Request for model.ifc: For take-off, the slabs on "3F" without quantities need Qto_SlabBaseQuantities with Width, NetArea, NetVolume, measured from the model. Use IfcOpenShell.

First a look at what the model holds.

```python
import ifcopenshell
import ifcopenshell.util.element
import ifcopenshell.util.unit

model = ifcopenshell.open("model.ifc")
print(model.schema)
for unit_type in ("LENGTHUNIT", "AREAUNIT", "VOLUMEUNIT"):
    print(unit_type, ifcopenshell.util.unit.calculate_unit_scale(model, unit_type))
storey = next(s for s in model.by_type("IfcBuildingStorey") if s.Name == "3F")
slabs = [e for e in ifcopenshell.util.element.get_decomposition(storey) if e.is_a("IfcSlab")]
for e in sorted(slabs, key=lambda e: e.id()):
    print(e.id(), e.is_a(), e.Name, list(ifcopenshell.util.element.get_psets(e, qtos_only=True)), sep=" | ")
```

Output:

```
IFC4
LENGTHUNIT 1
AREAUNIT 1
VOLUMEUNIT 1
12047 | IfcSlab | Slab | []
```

```python
import ifcopenshell
import ifcopenshell.api.pset
import ifcopenshell.geom
import ifcopenshell.util.element
import ifcopenshell.util.shape
import ifcopenshell.util.unit

model = ifcopenshell.open("model.ifc")
unit_scale = ifcopenshell.util.unit.calculate_unit_scale(model)
area_scale = ifcopenshell.util.unit.calculate_unit_scale(model, "AREAUNIT")
volume_scale = ifcopenshell.util.unit.calculate_unit_scale(model, "VOLUMEUNIT")
settings = ifcopenshell.geom.settings()

storey = next(s for s in model.by_type("IfcBuildingStorey") if s.Name == "3F")
slabs = [e for e in ifcopenshell.util.element.get_decomposition(storey) if e.is_a("IfcSlab")]

for e in sorted(slabs, key=lambda e: e.id()):
    if ifcopenshell.util.element.get_psets(e, qtos_only=True, should_inherit=False):
        continue
    # Geometry comes back in metres, in the element's own axes.
    shape = ifcopenshell.geom.create_shape(settings, e)
    values = {
        "Width": ifcopenshell.util.shape.get_z(shape.geometry) / unit_scale,
        "NetArea": ifcopenshell.util.shape.get_footprint_area(shape.geometry) / area_scale,
        "NetVolume": ifcopenshell.util.shape.get_volume(shape.geometry) / volume_scale,
    }
    qto = ifcopenshell.api.pset.add_qto(model, product=e, name="Qto_SlabBaseQuantities")
    ifcopenshell.api.pset.edit_qto(model, qto=qto, properties=values)
    print(e.id(), {k: round(v, 3) for k, v in values.items()})

model.write("model_rev.ifc")
```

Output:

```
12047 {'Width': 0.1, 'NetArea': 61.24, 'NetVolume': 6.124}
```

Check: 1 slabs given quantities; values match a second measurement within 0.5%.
